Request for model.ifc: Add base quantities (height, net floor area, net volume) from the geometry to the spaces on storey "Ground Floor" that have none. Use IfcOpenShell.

First a look at what the model holds.

```python
import ifcopenshell
import ifcopenshell.util.element
import ifcopenshell.util.unit

model = ifcopenshell.open("model.ifc")
print(model.schema)
for unit_type in ("LENGTHUNIT", "AREAUNIT", "VOLUMEUNIT"):
    print(unit_type, ifcopenshell.util.unit.calculate_unit_scale(model, unit_type))
storey = next(s for s in model.by_type("IfcBuildingStorey") if s.Name == "Ground Floor")
spaces = [e for e in ifcopenshell.util.element.get_decomposition(storey) if e.is_a("IfcSpace")]
for e in sorted(spaces, key=lambda e: e.id()):
    print(e.id(), e.is_a(), e.Name, list(ifcopenshell.util.element.get_psets(e, qtos_only=True)), sep=" | ")
```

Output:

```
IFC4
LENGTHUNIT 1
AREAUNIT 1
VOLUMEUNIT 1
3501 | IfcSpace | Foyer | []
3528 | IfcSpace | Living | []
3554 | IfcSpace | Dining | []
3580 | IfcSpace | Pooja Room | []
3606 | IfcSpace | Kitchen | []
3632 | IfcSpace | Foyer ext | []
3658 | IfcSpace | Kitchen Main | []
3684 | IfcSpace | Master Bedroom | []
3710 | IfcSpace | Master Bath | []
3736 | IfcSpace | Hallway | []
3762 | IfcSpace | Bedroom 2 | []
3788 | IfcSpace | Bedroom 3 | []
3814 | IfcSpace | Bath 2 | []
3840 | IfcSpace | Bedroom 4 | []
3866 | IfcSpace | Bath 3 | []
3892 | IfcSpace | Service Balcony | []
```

```python
import ifcopenshell
import ifcopenshell.api.pset
import ifcopenshell.geom
import ifcopenshell.util.element
import ifcopenshell.util.shape
import ifcopenshell.util.unit

model = ifcopenshell.open("model.ifc")
unit_scale = ifcopenshell.util.unit.calculate_unit_scale(model)
area_scale = ifcopenshell.util.unit.calculate_unit_scale(model, "AREAUNIT")
volume_scale = ifcopenshell.util.unit.calculate_unit_scale(model, "VOLUMEUNIT")
settings = ifcopenshell.geom.settings()

storey = next(s for s in model.by_type("IfcBuildingStorey") if s.Name == "Ground Floor")
spaces = [e for e in ifcopenshell.util.element.get_decomposition(storey) if e.is_a("IfcSpace")]

for e in sorted(spaces, key=lambda e: e.id()):
    if ifcopenshell.util.element.get_psets(e, qtos_only=True, should_inherit=False):
        continue
    # Geometry comes back in metres, in the element's own axes.
    shape = ifcopenshell.geom.create_shape(settings, e)
    values = {
        "Height": ifcopenshell.util.shape.get_z(shape.geometry) / unit_scale,
        "NetFloorArea": ifcopenshell.util.shape.get_footprint_area(shape.geometry) / area_scale,
        "NetVolume": ifcopenshell.util.shape.get_volume(shape.geometry) / volume_scale,
    }
    qto = ifcopenshell.api.pset.add_qto(model, product=e, name="Qto_SpaceBaseQuantities")
    ifcopenshell.api.pset.edit_qto(model, qto=qto, properties=values)
    print(e.id(), {k: round(v, 3) for k, v in values.items()})

model.write("model-out.ifc")
```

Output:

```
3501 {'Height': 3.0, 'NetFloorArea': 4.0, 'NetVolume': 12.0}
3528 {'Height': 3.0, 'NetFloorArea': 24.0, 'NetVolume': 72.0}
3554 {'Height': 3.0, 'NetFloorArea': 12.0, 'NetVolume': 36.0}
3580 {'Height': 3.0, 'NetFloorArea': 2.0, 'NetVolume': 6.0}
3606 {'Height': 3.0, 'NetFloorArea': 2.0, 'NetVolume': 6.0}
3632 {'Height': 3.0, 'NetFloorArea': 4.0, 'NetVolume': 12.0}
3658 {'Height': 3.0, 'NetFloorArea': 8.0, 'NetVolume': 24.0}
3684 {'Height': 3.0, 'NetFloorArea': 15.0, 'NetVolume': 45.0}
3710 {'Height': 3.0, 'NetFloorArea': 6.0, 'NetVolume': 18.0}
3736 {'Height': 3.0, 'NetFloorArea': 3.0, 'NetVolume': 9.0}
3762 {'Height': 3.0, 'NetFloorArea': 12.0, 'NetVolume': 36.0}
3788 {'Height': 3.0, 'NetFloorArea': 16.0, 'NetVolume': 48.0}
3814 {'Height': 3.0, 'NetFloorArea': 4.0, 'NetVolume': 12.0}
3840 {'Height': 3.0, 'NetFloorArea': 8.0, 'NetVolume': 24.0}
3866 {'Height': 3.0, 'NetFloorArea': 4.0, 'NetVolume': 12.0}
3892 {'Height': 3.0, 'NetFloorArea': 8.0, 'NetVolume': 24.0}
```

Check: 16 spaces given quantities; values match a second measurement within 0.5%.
